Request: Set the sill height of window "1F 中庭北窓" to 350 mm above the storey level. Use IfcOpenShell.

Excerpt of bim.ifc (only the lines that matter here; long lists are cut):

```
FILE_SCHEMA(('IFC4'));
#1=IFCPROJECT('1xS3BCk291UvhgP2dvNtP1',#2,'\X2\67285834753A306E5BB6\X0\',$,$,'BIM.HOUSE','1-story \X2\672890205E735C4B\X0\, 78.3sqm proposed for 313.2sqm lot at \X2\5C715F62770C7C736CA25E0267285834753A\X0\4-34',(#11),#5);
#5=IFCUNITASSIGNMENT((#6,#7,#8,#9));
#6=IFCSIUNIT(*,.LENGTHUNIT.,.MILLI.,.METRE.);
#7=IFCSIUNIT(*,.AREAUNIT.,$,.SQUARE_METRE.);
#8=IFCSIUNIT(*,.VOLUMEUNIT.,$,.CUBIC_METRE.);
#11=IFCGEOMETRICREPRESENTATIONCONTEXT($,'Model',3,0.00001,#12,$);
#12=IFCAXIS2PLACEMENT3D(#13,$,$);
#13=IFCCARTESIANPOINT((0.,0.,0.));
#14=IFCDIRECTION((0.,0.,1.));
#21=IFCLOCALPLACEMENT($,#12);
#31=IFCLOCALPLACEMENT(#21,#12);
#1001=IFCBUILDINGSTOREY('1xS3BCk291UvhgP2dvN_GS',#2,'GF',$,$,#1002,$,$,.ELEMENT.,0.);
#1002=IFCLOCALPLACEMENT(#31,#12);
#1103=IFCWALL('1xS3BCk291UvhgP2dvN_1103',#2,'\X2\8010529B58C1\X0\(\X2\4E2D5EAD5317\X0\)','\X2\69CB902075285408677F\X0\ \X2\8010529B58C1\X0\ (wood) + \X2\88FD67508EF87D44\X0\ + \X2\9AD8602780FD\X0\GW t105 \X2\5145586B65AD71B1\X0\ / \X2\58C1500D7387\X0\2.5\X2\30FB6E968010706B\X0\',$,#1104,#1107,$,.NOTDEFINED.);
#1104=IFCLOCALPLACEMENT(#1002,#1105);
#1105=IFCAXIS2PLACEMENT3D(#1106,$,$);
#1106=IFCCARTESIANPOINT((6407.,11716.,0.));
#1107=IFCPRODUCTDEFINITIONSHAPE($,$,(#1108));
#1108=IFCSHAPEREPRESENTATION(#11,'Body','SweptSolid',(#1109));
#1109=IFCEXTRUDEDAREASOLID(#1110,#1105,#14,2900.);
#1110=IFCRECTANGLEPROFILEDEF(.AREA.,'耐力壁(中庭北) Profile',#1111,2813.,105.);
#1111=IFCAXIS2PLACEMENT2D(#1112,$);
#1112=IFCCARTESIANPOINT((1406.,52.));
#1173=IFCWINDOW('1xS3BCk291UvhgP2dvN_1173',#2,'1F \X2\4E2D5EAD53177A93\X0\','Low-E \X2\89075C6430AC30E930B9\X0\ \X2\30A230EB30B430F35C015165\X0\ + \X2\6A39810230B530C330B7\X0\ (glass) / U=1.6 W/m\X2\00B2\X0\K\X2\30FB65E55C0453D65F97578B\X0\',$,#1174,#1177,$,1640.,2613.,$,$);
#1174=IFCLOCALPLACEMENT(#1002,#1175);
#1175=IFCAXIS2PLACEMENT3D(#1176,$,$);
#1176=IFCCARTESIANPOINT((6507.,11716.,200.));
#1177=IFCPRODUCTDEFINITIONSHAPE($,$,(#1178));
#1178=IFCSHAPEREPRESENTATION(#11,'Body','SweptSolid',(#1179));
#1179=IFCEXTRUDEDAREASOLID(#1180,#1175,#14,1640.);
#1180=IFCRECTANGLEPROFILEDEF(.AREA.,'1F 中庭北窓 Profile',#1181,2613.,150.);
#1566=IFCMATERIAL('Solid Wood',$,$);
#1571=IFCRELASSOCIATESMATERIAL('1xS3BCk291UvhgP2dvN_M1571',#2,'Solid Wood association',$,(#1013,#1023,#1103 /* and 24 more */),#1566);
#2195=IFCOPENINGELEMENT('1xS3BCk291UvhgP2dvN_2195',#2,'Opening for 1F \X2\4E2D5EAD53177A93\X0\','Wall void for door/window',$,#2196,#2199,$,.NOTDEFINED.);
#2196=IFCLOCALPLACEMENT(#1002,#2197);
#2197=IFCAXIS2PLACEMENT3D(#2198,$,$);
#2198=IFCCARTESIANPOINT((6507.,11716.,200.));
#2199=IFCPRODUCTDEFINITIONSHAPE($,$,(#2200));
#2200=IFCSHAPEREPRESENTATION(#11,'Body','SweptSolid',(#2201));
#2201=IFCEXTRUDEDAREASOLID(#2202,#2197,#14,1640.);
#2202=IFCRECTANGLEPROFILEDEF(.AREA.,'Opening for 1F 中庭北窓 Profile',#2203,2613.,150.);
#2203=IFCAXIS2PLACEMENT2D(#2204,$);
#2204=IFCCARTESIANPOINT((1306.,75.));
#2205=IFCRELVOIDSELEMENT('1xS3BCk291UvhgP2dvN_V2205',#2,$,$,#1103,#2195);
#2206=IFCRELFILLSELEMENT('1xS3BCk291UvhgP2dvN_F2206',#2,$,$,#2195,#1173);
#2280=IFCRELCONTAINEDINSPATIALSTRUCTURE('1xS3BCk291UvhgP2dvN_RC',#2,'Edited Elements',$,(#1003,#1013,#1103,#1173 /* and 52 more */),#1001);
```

```python
import numpy as np
import ifcopenshell
import ifcopenshell.api.geometry
import ifcopenshell.geom
import ifcopenshell.util.element
import ifcopenshell.util.placement
import ifcopenshell.util.shape
import ifcopenshell.util.unit

model = ifcopenshell.open("bim.ifc")
unit_scale = ifcopenshell.util.unit.calculate_unit_scale(model)

window = model.by_id(1173)
opening = window.FillsVoids[0].RelatingOpeningElement
storey = ifcopenshell.util.element.get_container(window, ifc_class="IfcBuildingStorey")
level = ifcopenshell.util.placement.get_local_placement(storey.ObjectPlacement)[2, 3]

# The opening's origin need not be at the sill, so measure its lowest point.
shape = ifcopenshell.geom.create_shape(ifcopenshell.geom.settings(), opening)
bottom = ifcopenshell.util.shape.get_shape_bottom_elevation(shape, shape.geometry) / unit_scale
dz = level + 0.35 / unit_scale - bottom

shift = np.array([0.0, 0.0, dz])
# The window is not placed relative to its opening, so move both.
for product in (opening, window):
    matrix = ifcopenshell.util.placement.get_local_placement(product.ObjectPlacement)
    matrix[:3, 3] += shift
    ifcopenshell.api.geometry.edit_object_placement(model, product=product, matrix=matrix, is_si=False)

print(f"moved by {dz * unit_scale:+.3f} m")

model.write("bim_v2.ifc")
```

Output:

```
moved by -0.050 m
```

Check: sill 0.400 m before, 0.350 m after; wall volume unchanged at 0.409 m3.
